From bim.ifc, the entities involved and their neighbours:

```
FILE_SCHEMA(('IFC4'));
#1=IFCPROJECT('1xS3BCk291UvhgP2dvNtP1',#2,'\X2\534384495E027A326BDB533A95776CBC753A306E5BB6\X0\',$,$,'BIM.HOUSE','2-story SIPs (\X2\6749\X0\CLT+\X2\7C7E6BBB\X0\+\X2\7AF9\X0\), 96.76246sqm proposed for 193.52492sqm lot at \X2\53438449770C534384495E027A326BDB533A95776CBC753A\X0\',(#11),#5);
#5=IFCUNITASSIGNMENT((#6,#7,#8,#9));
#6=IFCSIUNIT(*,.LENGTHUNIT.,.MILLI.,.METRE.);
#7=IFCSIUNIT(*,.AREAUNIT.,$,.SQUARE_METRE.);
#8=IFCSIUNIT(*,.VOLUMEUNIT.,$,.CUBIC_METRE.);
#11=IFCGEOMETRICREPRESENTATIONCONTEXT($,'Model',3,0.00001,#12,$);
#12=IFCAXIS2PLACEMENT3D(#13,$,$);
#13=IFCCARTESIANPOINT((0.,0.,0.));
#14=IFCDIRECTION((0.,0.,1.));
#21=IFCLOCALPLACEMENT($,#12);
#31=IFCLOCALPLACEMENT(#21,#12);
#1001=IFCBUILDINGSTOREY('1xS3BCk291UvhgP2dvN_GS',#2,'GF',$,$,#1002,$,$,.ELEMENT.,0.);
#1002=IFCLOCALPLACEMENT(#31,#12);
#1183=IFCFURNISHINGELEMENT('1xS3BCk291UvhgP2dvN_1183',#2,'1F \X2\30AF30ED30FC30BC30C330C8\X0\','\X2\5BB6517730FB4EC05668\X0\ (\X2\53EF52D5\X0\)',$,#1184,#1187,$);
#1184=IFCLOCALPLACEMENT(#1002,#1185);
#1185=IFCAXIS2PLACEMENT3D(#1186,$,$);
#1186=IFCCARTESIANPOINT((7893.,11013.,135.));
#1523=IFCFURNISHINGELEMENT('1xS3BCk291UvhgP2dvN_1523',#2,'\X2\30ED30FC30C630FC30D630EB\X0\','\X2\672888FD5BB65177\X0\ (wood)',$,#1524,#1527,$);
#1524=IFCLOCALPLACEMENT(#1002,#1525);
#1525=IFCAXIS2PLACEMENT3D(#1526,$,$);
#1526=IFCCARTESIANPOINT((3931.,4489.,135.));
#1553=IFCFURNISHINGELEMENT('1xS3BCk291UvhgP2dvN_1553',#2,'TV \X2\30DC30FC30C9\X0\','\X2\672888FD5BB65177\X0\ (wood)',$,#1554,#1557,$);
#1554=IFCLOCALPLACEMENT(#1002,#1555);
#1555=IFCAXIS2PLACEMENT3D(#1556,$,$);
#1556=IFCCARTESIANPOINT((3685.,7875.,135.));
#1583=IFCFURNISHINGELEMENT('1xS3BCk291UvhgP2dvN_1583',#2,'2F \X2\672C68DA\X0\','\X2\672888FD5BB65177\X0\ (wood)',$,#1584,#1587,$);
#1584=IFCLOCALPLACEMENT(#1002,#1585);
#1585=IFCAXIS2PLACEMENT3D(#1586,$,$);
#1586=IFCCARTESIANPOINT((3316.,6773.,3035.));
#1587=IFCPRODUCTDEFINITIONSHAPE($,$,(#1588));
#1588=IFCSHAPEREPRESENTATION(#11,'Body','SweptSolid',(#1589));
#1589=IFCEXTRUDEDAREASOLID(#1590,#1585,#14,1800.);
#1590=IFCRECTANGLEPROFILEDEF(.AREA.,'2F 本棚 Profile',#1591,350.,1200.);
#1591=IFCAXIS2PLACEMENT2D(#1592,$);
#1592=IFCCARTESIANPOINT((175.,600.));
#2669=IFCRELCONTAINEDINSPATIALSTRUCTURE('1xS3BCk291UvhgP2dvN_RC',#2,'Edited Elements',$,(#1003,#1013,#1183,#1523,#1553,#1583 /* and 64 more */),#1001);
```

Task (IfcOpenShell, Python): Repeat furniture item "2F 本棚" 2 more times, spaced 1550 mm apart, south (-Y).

```python
import numpy as np
import ifcopenshell
import ifcopenshell.api.geometry
import ifcopenshell.api.root
import ifcopenshell.util.element
import ifcopenshell.util.placement

model = ifcopenshell.open("bim.ifc")


def reuse_history(source, copy):
    """copy_class also copies each property set's owner history, people and application; keep the originals."""
    for rel in copy.IsDefinedBy:
        if rel.is_a("IfcRelDefinesByProperties") and (history := rel.RelatingPropertyDefinition.OwnerHistory):
            rel.RelatingPropertyDefinition.OwnerHistory = source.OwnerHistory
            ifcopenshell.util.element.remove_deep2(model, history)


source = model.by_guid("1xS3BCk291UvhgP2dvN_1583")
base = ifcopenshell.util.placement.get_local_placement(source.ObjectPlacement)
step = np.array([0.0, -1.0, 0.0]) * 1550.0

for i in range(1, 3):
    copy = ifcopenshell.api.root.copy_class(model, product=source)
    copy.Representation = ifcopenshell.util.element.copy_deep(
        model, source.Representation, exclude=["IfcGeometricRepresentationContext", "IfcRepresentationMap"]
    )
    reuse_history(source, copy)
    matrix = base.copy()
    matrix[:3, 3] += i * step
    print("added at", matrix[:3, 3].round(3) + 0.0)
    ifcopenshell.api.geometry.edit_object_placement(model, product=copy, matrix=matrix, is_si=False)

model.write("bim-out.ifc")
```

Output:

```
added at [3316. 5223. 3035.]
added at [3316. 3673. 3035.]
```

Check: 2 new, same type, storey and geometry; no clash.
